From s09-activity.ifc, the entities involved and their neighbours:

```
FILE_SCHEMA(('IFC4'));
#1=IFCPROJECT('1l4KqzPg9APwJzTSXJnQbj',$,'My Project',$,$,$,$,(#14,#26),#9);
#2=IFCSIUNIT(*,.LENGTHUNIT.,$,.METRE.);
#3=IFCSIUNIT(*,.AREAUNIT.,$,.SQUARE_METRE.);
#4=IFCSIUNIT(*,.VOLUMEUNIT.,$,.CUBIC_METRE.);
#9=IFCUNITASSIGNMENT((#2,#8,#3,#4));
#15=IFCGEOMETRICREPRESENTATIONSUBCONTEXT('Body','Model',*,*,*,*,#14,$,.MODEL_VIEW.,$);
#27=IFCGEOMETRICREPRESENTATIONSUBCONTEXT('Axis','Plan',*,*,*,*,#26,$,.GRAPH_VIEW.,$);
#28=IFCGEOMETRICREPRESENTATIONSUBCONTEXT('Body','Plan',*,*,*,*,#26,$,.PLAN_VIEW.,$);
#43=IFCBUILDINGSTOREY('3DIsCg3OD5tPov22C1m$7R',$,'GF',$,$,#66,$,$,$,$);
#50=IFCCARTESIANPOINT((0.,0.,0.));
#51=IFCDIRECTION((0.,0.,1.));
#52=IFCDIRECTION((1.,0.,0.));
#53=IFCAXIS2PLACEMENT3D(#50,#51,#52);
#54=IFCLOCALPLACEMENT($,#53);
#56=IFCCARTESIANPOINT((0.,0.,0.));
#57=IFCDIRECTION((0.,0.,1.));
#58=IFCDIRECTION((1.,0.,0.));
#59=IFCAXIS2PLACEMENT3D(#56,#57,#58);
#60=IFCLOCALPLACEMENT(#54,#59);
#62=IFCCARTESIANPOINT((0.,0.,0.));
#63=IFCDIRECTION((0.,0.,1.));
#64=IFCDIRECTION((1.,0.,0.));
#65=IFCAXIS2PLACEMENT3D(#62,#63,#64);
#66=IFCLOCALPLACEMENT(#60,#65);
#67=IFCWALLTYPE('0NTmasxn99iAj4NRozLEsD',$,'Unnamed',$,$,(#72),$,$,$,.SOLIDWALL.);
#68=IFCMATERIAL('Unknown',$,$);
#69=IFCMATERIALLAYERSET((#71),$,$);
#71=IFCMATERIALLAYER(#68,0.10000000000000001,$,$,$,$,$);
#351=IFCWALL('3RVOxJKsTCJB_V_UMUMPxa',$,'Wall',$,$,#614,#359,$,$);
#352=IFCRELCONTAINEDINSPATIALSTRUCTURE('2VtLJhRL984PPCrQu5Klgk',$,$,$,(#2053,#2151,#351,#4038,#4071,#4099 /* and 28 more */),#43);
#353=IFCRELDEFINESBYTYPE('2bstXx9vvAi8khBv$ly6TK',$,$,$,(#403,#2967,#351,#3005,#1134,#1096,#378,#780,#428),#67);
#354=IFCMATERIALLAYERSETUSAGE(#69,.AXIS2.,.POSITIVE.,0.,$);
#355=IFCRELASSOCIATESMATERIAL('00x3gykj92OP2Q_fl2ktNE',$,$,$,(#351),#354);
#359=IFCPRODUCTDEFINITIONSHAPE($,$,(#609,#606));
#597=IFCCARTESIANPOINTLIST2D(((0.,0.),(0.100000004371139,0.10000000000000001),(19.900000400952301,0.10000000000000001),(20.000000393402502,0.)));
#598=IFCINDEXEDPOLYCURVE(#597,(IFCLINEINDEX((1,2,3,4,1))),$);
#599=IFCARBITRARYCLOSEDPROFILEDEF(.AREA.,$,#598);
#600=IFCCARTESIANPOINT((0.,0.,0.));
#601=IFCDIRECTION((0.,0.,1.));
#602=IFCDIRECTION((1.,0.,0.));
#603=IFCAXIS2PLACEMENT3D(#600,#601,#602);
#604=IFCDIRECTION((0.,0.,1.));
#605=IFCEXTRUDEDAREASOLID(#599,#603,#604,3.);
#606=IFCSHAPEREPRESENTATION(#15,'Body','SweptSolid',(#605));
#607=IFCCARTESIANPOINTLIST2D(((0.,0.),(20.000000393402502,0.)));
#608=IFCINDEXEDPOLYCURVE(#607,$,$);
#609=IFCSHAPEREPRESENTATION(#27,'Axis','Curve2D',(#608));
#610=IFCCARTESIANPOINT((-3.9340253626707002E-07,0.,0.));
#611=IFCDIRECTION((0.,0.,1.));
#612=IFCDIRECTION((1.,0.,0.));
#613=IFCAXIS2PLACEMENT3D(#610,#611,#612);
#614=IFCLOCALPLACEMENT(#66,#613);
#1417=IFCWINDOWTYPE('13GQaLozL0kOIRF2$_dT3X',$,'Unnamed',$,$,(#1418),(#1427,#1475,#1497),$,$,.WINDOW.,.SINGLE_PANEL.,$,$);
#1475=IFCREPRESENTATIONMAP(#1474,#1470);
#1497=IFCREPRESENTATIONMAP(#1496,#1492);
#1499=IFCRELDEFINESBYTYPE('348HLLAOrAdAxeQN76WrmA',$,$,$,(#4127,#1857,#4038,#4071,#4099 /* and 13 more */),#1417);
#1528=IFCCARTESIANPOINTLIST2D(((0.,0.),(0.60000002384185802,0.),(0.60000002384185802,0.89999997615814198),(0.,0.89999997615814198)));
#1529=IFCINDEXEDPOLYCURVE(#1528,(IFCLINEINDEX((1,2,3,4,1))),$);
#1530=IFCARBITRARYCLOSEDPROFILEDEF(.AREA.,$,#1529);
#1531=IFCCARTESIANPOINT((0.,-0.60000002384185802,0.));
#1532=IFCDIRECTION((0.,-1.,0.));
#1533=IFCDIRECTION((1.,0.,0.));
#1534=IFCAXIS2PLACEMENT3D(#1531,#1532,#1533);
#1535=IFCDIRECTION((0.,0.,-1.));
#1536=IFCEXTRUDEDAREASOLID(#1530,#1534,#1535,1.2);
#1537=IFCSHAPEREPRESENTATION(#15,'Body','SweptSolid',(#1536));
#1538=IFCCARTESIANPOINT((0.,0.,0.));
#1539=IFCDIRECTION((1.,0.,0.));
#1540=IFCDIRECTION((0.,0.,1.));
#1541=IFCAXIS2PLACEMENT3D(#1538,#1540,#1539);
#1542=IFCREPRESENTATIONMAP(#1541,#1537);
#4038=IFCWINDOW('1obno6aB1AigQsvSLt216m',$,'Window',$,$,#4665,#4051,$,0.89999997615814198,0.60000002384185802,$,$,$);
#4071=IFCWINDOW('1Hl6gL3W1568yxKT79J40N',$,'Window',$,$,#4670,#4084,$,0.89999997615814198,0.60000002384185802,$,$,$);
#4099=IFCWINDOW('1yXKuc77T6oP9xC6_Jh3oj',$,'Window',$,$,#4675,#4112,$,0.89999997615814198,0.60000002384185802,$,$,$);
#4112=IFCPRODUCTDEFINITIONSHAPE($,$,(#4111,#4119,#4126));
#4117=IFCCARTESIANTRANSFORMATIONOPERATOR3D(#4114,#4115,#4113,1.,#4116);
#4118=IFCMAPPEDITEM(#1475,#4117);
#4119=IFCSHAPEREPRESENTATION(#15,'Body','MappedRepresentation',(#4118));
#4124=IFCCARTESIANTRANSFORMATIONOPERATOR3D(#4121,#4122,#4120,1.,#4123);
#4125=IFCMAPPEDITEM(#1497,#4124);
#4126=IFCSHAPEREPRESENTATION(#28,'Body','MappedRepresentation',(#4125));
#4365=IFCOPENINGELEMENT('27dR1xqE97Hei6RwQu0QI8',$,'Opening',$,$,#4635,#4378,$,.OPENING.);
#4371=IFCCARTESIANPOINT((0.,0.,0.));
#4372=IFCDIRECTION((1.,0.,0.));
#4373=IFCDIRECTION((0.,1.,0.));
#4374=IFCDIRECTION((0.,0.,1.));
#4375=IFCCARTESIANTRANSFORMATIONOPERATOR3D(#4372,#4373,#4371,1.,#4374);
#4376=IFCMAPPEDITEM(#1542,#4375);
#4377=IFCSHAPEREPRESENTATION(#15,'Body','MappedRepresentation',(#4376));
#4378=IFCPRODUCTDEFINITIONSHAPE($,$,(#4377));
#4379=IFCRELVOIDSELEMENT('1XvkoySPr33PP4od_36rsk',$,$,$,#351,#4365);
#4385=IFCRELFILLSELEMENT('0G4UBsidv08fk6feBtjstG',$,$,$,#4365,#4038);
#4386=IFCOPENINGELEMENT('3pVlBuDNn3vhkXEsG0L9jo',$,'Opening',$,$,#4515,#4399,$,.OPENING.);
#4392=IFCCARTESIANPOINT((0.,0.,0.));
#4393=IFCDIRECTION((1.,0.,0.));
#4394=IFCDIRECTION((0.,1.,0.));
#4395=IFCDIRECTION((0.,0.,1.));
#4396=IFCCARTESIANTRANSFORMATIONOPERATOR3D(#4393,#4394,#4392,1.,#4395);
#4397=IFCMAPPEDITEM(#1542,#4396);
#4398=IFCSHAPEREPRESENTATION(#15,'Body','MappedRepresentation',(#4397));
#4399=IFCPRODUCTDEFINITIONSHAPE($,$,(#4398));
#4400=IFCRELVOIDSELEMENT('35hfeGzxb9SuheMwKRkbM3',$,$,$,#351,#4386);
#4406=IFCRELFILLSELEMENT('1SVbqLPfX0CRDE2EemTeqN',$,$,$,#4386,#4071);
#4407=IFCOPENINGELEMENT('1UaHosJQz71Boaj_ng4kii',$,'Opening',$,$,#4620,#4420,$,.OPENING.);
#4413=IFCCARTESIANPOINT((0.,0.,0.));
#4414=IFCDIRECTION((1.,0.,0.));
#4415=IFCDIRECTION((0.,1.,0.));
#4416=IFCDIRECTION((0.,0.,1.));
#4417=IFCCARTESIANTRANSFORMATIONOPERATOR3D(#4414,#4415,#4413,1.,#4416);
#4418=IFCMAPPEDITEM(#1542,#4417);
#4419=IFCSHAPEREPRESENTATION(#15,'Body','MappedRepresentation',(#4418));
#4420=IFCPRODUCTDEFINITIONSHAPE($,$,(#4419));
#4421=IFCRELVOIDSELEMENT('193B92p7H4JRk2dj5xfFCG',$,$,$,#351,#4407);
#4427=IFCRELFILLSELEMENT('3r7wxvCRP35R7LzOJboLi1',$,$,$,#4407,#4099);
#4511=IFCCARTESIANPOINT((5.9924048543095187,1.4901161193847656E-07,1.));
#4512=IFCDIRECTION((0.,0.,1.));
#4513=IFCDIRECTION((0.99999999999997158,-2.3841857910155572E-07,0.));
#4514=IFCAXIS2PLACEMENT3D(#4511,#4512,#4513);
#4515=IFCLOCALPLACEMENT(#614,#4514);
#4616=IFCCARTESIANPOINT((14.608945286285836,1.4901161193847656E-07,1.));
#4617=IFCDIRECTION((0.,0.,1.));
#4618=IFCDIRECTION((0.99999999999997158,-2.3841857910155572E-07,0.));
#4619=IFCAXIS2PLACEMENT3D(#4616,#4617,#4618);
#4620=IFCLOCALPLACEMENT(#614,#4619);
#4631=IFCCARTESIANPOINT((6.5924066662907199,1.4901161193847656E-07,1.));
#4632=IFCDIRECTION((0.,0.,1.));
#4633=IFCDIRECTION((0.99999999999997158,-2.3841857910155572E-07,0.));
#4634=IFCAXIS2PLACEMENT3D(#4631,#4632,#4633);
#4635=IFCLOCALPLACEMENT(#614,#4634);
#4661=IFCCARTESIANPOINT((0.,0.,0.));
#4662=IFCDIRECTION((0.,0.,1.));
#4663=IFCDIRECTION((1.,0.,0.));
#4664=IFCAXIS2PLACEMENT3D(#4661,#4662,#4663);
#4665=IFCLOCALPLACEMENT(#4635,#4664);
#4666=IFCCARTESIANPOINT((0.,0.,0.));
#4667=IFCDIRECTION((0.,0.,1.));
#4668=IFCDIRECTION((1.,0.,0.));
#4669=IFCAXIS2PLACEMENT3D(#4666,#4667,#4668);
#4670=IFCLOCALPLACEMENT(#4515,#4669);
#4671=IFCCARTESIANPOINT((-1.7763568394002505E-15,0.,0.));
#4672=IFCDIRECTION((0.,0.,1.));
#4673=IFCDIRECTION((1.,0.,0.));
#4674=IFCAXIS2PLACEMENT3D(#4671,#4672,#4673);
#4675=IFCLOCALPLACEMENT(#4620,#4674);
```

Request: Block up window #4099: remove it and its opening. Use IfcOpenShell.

```python
import ifcopenshell
import ifcopenshell.api.feature
import ifcopenshell.api.root
import ifcopenshell.geom
import ifcopenshell.util.shape

model = ifcopenshell.open("s09-activity.ifc")
settings = ifcopenshell.geom.settings()


def volume(element):
    """Net volume in cubic metres, openings subtracted."""
    shape = ifcopenshell.geom.create_shape(settings, element)
    return ifcopenshell.util.shape.get_volume(shape.geometry)


window = model.by_guid("1yXKuc77T6oP9xC6_Jh3oj")
opening = window.FillsVoids[0].RelatingOpeningElement
wall = opening.VoidsElements[0].RelatingBuildingElement
before = volume(wall)

ifcopenshell.api.root.remove_product(model, product=window)
ifcopenshell.api.feature.remove_feature(model, feature=opening)

after = volume(wall)

print(f"wall volume {before:.3f} -> {after:.3f} m3")

model.write("s09-activity_v2.ifc")
```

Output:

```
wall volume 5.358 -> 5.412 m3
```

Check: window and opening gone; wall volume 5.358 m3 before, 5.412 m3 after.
